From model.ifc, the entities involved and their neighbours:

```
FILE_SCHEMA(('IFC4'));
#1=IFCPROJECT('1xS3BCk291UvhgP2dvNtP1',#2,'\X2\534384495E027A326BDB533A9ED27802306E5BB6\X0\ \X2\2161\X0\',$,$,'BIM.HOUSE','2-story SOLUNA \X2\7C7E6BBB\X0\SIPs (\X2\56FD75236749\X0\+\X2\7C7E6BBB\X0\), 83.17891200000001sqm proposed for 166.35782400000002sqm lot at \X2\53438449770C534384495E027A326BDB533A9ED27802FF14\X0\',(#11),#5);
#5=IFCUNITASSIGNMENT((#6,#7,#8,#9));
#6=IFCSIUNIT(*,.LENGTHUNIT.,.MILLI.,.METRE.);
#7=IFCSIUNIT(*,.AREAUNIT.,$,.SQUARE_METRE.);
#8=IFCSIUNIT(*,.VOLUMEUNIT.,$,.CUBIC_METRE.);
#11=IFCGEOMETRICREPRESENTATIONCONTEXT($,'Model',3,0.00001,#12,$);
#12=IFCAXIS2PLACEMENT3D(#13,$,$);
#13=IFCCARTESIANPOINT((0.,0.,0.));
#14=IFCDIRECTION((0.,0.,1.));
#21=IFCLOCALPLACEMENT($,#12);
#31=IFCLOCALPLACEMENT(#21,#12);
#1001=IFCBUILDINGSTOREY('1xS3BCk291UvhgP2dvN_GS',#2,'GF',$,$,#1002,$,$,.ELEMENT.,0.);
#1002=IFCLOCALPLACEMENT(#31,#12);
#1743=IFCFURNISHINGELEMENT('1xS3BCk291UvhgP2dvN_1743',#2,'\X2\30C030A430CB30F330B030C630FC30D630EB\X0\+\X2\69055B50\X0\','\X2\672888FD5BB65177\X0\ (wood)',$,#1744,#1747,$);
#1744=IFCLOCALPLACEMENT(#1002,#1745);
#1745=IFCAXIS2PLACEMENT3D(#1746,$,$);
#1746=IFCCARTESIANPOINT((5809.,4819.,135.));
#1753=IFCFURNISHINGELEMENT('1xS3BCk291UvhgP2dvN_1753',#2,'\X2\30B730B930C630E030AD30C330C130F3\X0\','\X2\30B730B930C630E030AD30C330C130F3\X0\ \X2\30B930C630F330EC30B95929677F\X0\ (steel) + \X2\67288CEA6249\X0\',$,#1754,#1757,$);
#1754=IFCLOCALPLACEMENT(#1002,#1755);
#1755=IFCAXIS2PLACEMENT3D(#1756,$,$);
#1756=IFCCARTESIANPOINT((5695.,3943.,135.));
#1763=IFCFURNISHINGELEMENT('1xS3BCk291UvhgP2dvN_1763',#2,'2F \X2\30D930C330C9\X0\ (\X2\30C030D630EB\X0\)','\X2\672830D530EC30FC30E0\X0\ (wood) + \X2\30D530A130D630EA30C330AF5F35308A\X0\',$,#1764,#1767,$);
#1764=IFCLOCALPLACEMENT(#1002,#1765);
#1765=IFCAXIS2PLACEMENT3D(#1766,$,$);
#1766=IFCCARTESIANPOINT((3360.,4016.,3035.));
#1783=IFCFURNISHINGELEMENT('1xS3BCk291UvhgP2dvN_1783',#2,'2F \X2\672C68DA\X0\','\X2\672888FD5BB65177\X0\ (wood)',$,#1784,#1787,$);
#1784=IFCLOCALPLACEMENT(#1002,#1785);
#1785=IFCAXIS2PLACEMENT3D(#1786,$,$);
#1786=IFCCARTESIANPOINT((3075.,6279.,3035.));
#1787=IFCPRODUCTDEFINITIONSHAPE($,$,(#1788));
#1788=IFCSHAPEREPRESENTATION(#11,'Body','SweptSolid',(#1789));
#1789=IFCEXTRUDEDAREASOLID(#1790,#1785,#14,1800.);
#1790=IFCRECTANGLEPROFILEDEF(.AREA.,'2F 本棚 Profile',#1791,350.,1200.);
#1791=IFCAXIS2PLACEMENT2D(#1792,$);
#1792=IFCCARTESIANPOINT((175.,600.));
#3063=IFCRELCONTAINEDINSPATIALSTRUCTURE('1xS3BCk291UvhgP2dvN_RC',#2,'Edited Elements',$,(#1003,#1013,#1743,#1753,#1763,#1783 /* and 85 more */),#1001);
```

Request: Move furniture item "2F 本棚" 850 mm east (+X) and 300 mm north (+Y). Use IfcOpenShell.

```python
import ifcopenshell
import ifcopenshell.api.geometry
import ifcopenshell.util.placement

model = ifcopenshell.open("model.ifc")

item = model.by_guid("1xS3BCk291UvhgP2dvN_1783")
matrix = ifcopenshell.util.placement.get_local_placement(item.ObjectPlacement)
matrix[0, 3] += 850.0
matrix[1, 3] += 300.0
ifcopenshell.api.geometry.edit_object_placement(model, product=item, matrix=matrix, is_si=False)

print(ifcopenshell.util.placement.get_local_placement(item.ObjectPlacement).round(3) + 0.0)

model.write("model_updated.ifc")
```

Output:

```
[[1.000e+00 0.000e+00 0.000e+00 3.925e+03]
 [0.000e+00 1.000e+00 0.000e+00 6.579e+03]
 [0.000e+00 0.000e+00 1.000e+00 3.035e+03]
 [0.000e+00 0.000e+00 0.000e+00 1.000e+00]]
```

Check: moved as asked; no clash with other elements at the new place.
